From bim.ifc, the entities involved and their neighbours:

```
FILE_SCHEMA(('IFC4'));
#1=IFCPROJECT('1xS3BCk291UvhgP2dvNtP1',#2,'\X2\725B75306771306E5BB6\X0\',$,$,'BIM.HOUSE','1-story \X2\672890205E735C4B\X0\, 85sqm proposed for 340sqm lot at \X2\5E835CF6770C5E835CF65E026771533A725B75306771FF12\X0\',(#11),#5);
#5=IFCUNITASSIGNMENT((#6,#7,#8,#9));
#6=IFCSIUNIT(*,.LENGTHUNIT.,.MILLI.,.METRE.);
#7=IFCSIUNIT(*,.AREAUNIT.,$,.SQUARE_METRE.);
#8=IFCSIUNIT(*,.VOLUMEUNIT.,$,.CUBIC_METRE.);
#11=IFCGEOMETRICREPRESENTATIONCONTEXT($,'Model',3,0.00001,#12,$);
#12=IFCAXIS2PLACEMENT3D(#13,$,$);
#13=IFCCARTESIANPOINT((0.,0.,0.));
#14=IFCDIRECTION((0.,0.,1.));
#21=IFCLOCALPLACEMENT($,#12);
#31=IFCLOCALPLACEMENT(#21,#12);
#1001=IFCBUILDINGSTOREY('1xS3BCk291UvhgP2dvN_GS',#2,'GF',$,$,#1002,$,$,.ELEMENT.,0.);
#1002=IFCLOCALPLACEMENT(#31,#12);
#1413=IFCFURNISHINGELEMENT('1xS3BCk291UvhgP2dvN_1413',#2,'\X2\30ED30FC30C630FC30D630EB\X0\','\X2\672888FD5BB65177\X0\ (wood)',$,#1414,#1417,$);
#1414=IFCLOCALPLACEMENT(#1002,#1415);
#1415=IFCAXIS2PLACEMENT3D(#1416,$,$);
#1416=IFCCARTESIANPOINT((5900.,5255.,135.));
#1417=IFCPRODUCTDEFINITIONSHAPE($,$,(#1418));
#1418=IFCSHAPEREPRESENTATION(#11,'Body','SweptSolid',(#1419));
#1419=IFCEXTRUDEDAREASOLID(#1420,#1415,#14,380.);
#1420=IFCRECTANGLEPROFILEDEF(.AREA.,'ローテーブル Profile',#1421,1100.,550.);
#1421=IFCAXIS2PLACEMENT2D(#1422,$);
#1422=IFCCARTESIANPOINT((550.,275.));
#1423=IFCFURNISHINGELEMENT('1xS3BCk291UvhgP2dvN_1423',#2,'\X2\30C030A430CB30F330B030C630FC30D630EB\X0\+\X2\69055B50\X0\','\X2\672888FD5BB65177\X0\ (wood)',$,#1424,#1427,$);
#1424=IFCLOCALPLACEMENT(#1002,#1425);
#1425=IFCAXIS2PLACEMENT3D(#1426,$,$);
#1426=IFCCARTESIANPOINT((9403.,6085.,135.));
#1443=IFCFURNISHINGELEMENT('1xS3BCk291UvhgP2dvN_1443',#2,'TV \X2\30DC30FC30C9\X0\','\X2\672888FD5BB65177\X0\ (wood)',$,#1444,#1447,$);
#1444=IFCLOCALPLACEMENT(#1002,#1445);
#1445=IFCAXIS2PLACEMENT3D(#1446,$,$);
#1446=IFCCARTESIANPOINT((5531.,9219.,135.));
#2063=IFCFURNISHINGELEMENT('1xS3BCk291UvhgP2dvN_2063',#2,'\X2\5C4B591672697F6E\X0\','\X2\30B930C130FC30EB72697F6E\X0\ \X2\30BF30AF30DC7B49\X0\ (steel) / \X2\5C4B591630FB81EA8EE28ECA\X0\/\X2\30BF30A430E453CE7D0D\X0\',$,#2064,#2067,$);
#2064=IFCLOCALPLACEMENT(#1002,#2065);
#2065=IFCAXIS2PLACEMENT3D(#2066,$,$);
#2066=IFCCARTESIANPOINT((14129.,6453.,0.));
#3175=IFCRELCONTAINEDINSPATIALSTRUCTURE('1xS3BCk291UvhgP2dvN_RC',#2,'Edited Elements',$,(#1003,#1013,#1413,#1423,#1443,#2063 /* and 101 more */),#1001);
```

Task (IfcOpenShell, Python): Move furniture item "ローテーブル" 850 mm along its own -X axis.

```python
import ifcopenshell
import ifcopenshell.api.geometry
import ifcopenshell.util.placement
import ifcopenshell.util.unit

model = ifcopenshell.open("bim.ifc")
unit_scale = ifcopenshell.util.unit.calculate_unit_scale(model)

item = model.by_guid("1xS3BCk291UvhgP2dvN_1413")
matrix = ifcopenshell.util.placement.get_local_placement(item.ObjectPlacement)
matrix[:3, 3] -= matrix[:3, 0] * 0.85 / unit_scale
ifcopenshell.api.geometry.edit_object_placement(model, product=item, matrix=matrix, is_si=False)

print(ifcopenshell.util.placement.get_local_placement(item.ObjectPlacement).round(3) + 0.0)

model.write("bim_updated.ifc")
```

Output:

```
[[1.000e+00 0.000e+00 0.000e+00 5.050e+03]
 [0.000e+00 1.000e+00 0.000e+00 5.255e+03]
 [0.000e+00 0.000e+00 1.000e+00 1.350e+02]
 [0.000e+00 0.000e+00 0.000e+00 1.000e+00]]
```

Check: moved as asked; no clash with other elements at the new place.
